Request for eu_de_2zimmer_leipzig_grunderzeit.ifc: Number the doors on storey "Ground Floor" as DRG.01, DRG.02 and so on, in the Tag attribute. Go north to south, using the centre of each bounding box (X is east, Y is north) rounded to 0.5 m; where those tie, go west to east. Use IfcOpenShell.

First a look at what the model holds.

```python
import ifcopenshell
import ifcopenshell.util.element
import ifcopenshell.util.placement

model = ifcopenshell.open("eu_de_2zimmer_leipzig_grunderzeit.ifc")
print(model.schema)
storey = next(s for s in model.by_type("IfcBuildingStorey") if s.Name == "Ground Floor")
doors = [e for e in ifcopenshell.util.element.get_decomposition(storey) if e.is_a("IfcDoor")]
for e in sorted(doors, key=lambda e: e.id()):
    origin = ifcopenshell.util.placement.get_local_placement(e.ObjectPlacement)[:3, 3]
    print(e.id(), e.Tag, e.Name, origin.round(2) + 0.0, sep=" | ")
```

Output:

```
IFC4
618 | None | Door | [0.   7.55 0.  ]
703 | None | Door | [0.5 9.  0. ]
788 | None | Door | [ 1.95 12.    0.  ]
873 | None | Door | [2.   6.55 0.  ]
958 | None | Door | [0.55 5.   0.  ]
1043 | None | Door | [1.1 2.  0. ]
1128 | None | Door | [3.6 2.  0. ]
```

```python
import ifcopenshell
import ifcopenshell.geom
import ifcopenshell.util.element
import ifcopenshell.util.shape

model = ifcopenshell.open("eu_de_2zimmer_leipzig_grunderzeit.ifc")
settings = ifcopenshell.geom.settings()
settings.set("use-world-coords", True)


def centre(element):
    shape = ifcopenshell.geom.create_shape(settings, element)
    return ifcopenshell.util.shape.get_bbox_centroid(shape.geometry)


storey = next(s for s in model.by_type("IfcBuildingStorey") if s.Name == "Ground Floor")
doors = [e for e in ifcopenshell.util.element.get_decomposition(storey) if e.is_a("IfcDoor")]

# Insertion points can sit at a corner or the storey origin, so sort by the geometry (in metres).
centres = {e: centre(e) for e in doors}
doors.sort(key=lambda e: (-round(centres[e][1] / 0.5), centres[e][0]))

for i, e in enumerate(doors, start=1):
    number = f"DRG.{i:02d}"
    e.Tag = number
    print(e.id(), number)

model.write("eu_de_2zimmer_leipzig_grunderzeit_edited.ifc")
```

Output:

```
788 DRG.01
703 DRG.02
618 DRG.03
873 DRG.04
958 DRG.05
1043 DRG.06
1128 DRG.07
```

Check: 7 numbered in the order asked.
